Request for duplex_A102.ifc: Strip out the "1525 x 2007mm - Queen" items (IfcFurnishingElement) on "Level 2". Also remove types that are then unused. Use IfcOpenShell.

First a look at what the model holds.

```python
import ifcopenshell
import ifcopenshell.util.element

model = ifcopenshell.open("duplex_A102.ifc")
print(model.schema)
storey = next(s for s in model.by_type("IfcBuildingStorey") if s.Name == "Level 2")
furniture = [e for e in ifcopenshell.util.element.get_decomposition(storey) if e.is_a("IfcFurnishingElement")]
seen = {}
for e in furniture:
    element_type = ifcopenshell.util.element.get_type(e)
    name = element_type.Name if element_type not in (None, e) else None
    seen[name] = seen.get(name, 0) + 1
for name, count in sorted(seen.items(), key=str):
    print(count, "x", name)
```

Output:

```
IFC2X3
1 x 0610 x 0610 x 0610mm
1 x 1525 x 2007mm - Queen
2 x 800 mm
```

```python
import ifcopenshell
import ifcopenshell.api.root
import ifcopenshell.util.element

model = ifcopenshell.open("duplex_A102.ifc")

storey = next(s for s in model.by_type("IfcBuildingStorey") if s.Name == "Level 2")
furniture = [e for e in ifcopenshell.util.element.get_decomposition(storey) if e.is_a("IfcFurnishingElement")]
targets = [e for e in furniture if (t := ifcopenshell.util.element.get_type(e)) not in (None, e) and t.Name == "1525 x 2007mm - Queen"]
types = {ifcopenshell.util.element.get_type(e) for e in targets} - {None, *targets}

for e in targets:
    ifcopenshell.api.root.remove_product(model, product=e)
print(len(targets), "removed")

unused = [t for t in types if not ifcopenshell.util.element.get_types(t)]
for t in unused:
    ifcopenshell.api.root.remove_product(model, product=t)
print(len(unused), "unused types removed")

model.write("duplex_A102-out.ifc")
```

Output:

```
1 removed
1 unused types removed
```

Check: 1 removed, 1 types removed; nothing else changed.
